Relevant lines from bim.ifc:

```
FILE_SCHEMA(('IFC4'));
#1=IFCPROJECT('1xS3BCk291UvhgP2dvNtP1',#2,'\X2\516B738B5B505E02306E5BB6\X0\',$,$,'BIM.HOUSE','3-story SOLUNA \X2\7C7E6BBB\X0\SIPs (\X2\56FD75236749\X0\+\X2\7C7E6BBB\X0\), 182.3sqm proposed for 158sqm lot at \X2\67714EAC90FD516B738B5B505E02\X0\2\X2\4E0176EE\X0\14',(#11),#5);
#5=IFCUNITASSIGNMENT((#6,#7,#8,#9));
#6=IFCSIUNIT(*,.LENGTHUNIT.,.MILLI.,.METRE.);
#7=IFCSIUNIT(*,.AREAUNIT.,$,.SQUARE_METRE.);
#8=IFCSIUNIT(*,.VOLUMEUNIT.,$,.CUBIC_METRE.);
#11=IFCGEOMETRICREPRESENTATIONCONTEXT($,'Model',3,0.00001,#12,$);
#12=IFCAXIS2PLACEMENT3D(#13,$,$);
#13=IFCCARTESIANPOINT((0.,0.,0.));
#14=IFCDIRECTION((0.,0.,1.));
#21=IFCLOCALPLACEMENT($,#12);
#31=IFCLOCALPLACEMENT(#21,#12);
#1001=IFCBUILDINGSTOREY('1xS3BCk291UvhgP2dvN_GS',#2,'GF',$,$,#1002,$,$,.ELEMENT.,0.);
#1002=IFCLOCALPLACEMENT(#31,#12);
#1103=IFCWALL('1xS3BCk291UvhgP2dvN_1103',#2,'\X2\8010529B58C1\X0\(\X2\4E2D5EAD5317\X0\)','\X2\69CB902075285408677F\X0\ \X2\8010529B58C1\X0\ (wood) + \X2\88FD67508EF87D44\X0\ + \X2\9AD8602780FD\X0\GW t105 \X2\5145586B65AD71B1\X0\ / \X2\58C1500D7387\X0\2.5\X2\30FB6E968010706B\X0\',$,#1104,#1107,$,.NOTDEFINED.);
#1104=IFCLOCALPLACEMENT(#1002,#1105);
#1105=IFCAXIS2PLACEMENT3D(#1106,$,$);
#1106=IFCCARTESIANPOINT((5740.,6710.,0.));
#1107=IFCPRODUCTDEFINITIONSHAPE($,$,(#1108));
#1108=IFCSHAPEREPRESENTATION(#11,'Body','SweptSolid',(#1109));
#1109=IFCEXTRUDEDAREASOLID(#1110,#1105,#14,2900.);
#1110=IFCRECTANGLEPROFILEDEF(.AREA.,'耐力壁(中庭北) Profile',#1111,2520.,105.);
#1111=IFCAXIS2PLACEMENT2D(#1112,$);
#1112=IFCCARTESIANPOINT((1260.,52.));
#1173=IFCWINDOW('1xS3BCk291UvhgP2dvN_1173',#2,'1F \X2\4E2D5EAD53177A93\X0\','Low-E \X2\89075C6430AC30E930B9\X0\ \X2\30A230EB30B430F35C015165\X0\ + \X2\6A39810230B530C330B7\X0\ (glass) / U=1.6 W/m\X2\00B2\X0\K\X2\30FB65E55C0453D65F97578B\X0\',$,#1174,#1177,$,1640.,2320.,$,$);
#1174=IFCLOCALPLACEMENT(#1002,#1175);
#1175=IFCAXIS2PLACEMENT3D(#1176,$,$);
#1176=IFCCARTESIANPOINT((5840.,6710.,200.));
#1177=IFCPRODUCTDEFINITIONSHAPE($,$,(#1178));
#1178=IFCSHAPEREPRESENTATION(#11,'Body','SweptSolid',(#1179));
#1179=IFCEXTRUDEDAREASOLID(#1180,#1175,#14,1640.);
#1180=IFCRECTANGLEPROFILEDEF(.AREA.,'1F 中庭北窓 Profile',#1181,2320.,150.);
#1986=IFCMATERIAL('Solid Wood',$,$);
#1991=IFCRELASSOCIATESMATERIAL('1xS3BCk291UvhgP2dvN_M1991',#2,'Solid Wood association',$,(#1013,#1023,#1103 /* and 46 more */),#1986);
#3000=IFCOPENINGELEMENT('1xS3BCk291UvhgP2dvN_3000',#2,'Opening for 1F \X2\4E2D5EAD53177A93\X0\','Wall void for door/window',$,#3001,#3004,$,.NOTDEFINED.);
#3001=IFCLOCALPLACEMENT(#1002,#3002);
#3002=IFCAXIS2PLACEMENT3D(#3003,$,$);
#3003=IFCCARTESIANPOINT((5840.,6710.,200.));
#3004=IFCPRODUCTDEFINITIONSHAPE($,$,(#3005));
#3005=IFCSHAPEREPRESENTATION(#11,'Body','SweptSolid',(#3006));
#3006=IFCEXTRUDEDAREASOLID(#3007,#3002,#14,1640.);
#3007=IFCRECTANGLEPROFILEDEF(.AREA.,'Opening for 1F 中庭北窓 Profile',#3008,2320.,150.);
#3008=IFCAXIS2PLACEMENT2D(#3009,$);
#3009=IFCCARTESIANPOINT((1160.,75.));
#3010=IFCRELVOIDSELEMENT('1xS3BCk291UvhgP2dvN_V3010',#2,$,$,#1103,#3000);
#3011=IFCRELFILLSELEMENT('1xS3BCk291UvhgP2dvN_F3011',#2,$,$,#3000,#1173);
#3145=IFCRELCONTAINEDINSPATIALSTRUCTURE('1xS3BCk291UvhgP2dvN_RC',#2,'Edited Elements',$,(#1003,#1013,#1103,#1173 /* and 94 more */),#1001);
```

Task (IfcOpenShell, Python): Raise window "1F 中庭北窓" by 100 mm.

```python
import numpy as np
import ifcopenshell
import ifcopenshell.api.geometry
import ifcopenshell.util.placement
import ifcopenshell.util.unit

model = ifcopenshell.open("bim.ifc")
unit_scale = ifcopenshell.util.unit.calculate_unit_scale(model)

window = model.by_guid("1xS3BCk291UvhgP2dvN_1173")
opening = window.FillsVoids[0].RelatingOpeningElement
dz = 0.1 / unit_scale

shift = np.array([0.0, 0.0, dz])
# The window is not placed relative to its opening, so move both.
for product in (opening, window):
    matrix = ifcopenshell.util.placement.get_local_placement(product.ObjectPlacement)
    matrix[:3, 3] += shift
    ifcopenshell.api.geometry.edit_object_placement(model, product=product, matrix=matrix, is_si=False)

print(f"moved by {dz * unit_scale:+.3f} m")

model.write("bim_updated.ifc")
```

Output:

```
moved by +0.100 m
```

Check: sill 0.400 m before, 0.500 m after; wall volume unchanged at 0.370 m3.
